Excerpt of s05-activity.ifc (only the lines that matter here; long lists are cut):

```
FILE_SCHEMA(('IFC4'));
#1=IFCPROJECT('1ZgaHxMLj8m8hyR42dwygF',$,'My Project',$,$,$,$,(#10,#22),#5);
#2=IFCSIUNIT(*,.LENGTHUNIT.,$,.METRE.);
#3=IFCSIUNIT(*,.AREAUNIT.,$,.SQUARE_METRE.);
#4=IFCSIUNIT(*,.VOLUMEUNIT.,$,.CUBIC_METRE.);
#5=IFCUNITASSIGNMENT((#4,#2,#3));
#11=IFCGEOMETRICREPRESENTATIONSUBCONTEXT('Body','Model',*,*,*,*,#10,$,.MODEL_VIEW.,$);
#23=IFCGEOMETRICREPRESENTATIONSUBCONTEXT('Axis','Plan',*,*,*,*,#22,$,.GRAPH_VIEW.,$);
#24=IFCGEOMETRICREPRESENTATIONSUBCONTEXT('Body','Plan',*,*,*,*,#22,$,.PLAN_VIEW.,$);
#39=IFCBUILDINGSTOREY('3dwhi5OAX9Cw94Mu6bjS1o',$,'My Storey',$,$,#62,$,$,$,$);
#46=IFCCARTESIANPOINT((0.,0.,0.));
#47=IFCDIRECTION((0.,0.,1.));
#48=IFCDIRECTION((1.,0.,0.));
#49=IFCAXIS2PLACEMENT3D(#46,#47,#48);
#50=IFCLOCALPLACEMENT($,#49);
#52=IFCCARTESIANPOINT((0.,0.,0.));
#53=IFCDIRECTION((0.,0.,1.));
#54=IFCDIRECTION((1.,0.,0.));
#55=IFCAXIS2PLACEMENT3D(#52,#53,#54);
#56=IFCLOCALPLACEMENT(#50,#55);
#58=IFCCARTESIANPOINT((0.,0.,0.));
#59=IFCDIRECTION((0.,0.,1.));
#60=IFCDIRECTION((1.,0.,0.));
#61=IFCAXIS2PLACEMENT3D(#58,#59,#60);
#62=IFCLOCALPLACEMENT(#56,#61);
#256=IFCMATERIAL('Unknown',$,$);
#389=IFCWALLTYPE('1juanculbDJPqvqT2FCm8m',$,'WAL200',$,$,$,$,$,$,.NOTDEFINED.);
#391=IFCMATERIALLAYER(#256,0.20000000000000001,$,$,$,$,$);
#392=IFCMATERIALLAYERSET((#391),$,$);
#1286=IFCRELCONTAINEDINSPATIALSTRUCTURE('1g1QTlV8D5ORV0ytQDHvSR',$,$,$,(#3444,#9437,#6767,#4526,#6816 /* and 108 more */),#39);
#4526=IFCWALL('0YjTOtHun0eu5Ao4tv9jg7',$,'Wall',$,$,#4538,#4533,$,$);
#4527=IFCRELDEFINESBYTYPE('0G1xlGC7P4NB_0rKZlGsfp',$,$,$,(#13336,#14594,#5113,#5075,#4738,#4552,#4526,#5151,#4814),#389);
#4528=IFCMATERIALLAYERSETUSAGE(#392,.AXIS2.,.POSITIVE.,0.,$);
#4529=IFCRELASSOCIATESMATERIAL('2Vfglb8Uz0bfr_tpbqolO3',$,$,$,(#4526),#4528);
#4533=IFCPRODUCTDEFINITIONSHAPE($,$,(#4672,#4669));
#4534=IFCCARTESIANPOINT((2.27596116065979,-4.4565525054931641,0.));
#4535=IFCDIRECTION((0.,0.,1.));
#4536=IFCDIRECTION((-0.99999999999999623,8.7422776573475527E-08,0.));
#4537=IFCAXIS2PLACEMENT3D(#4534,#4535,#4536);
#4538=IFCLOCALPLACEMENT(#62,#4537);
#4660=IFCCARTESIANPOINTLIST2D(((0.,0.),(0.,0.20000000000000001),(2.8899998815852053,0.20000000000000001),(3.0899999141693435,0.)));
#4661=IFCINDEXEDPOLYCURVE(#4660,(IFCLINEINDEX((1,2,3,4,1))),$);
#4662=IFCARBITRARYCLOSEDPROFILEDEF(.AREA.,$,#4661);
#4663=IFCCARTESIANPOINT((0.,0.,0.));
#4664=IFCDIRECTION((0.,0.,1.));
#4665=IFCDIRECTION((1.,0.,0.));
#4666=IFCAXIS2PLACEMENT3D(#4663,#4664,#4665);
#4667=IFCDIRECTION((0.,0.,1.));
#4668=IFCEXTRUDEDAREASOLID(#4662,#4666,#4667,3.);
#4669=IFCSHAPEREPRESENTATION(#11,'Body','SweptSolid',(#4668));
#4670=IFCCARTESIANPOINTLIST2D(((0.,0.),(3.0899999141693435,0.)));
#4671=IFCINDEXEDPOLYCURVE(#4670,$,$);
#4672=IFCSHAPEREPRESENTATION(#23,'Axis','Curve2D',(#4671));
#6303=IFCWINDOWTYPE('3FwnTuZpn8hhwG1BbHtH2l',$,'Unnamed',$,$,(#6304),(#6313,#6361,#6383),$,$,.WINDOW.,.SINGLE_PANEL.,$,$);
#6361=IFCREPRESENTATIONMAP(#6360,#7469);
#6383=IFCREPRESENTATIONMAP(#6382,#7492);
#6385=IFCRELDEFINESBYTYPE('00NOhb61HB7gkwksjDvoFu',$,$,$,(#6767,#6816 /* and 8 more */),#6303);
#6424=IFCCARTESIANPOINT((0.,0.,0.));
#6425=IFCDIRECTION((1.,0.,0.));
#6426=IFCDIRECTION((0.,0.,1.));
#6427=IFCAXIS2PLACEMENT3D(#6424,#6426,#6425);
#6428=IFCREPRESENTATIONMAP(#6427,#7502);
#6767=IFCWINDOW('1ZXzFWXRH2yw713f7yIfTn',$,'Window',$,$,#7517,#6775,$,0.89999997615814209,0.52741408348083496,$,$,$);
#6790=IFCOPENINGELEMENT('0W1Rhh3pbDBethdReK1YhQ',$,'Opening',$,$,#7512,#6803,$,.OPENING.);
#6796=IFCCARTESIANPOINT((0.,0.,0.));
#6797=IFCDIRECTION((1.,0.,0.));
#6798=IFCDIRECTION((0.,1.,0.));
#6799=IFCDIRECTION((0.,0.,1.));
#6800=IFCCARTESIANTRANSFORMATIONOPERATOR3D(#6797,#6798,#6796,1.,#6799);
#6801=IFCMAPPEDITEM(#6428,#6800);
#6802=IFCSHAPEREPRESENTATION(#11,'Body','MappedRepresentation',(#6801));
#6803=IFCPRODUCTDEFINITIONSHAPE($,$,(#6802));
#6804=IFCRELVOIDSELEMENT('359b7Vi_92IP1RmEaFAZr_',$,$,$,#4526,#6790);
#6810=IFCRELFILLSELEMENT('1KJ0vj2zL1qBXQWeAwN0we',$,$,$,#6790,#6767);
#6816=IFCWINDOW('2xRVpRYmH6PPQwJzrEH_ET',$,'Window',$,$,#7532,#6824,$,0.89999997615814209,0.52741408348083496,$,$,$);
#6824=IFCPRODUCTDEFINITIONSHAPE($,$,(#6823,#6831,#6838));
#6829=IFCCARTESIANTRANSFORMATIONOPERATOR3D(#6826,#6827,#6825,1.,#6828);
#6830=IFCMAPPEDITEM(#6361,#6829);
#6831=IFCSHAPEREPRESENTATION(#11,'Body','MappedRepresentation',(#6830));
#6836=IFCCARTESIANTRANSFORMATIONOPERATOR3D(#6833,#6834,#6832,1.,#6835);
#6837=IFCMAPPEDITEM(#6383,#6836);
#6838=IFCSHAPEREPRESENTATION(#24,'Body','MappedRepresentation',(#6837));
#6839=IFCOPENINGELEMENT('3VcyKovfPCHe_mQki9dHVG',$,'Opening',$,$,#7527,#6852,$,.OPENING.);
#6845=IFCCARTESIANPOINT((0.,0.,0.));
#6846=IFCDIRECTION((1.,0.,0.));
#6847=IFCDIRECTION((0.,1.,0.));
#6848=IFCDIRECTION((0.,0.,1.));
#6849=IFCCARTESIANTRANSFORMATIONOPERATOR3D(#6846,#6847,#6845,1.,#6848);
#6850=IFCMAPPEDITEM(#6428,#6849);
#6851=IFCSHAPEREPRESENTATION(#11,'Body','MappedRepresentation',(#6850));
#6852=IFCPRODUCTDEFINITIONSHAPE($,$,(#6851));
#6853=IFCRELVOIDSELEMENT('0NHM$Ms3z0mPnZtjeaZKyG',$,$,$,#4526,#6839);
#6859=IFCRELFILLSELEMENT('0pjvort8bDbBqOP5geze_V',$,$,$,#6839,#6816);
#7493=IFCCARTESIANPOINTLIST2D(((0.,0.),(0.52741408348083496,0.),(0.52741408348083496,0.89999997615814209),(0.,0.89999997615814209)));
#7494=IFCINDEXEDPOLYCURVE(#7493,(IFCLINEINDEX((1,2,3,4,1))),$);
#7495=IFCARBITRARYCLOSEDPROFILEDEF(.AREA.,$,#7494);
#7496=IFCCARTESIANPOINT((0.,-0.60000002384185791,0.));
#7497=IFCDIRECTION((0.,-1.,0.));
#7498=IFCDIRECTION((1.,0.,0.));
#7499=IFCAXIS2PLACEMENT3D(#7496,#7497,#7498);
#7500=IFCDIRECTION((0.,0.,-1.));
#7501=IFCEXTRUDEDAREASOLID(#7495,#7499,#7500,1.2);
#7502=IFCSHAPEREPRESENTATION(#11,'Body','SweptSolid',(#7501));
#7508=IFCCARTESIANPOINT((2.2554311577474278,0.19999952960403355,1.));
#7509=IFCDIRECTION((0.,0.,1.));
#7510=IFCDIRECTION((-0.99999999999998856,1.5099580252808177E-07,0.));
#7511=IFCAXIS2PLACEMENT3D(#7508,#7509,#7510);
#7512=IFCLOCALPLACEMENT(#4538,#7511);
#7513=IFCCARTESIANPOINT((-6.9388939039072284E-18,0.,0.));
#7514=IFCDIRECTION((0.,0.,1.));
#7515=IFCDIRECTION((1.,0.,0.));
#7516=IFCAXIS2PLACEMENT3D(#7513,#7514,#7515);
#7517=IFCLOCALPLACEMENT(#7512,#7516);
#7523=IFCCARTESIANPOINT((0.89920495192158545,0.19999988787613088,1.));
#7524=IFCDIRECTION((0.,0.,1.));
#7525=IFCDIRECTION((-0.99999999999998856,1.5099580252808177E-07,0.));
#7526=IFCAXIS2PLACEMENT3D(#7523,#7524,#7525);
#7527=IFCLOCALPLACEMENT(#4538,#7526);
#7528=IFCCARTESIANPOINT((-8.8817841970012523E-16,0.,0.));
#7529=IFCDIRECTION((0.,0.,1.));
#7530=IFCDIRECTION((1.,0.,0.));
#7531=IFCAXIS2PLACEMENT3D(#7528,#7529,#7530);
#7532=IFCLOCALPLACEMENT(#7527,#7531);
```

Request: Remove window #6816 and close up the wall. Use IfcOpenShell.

```python
import ifcopenshell
import ifcopenshell.api.feature
import ifcopenshell.api.root
import ifcopenshell.geom
import ifcopenshell.util.shape

model = ifcopenshell.open("s05-activity.ifc")
settings = ifcopenshell.geom.settings()


def volume(element):
    """Net volume in cubic metres, openings subtracted."""
    shape = ifcopenshell.geom.create_shape(settings, element)
    return ifcopenshell.util.shape.get_volume(shape.geometry)


window = model.by_id(6816)
opening = window.FillsVoids[0].RelatingOpeningElement
wall = opening.VoidsElements[0].RelatingBuildingElement
before = volume(wall)

ifcopenshell.api.root.remove_product(model, product=window)
ifcopenshell.api.feature.remove_feature(model, feature=opening)

after = volume(wall)

print(f"wall volume {before:.3f} -> {after:.3f} m3")

model.write("s05-activity_updated.ifc")
```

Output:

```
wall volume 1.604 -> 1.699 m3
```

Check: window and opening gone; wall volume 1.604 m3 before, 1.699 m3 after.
